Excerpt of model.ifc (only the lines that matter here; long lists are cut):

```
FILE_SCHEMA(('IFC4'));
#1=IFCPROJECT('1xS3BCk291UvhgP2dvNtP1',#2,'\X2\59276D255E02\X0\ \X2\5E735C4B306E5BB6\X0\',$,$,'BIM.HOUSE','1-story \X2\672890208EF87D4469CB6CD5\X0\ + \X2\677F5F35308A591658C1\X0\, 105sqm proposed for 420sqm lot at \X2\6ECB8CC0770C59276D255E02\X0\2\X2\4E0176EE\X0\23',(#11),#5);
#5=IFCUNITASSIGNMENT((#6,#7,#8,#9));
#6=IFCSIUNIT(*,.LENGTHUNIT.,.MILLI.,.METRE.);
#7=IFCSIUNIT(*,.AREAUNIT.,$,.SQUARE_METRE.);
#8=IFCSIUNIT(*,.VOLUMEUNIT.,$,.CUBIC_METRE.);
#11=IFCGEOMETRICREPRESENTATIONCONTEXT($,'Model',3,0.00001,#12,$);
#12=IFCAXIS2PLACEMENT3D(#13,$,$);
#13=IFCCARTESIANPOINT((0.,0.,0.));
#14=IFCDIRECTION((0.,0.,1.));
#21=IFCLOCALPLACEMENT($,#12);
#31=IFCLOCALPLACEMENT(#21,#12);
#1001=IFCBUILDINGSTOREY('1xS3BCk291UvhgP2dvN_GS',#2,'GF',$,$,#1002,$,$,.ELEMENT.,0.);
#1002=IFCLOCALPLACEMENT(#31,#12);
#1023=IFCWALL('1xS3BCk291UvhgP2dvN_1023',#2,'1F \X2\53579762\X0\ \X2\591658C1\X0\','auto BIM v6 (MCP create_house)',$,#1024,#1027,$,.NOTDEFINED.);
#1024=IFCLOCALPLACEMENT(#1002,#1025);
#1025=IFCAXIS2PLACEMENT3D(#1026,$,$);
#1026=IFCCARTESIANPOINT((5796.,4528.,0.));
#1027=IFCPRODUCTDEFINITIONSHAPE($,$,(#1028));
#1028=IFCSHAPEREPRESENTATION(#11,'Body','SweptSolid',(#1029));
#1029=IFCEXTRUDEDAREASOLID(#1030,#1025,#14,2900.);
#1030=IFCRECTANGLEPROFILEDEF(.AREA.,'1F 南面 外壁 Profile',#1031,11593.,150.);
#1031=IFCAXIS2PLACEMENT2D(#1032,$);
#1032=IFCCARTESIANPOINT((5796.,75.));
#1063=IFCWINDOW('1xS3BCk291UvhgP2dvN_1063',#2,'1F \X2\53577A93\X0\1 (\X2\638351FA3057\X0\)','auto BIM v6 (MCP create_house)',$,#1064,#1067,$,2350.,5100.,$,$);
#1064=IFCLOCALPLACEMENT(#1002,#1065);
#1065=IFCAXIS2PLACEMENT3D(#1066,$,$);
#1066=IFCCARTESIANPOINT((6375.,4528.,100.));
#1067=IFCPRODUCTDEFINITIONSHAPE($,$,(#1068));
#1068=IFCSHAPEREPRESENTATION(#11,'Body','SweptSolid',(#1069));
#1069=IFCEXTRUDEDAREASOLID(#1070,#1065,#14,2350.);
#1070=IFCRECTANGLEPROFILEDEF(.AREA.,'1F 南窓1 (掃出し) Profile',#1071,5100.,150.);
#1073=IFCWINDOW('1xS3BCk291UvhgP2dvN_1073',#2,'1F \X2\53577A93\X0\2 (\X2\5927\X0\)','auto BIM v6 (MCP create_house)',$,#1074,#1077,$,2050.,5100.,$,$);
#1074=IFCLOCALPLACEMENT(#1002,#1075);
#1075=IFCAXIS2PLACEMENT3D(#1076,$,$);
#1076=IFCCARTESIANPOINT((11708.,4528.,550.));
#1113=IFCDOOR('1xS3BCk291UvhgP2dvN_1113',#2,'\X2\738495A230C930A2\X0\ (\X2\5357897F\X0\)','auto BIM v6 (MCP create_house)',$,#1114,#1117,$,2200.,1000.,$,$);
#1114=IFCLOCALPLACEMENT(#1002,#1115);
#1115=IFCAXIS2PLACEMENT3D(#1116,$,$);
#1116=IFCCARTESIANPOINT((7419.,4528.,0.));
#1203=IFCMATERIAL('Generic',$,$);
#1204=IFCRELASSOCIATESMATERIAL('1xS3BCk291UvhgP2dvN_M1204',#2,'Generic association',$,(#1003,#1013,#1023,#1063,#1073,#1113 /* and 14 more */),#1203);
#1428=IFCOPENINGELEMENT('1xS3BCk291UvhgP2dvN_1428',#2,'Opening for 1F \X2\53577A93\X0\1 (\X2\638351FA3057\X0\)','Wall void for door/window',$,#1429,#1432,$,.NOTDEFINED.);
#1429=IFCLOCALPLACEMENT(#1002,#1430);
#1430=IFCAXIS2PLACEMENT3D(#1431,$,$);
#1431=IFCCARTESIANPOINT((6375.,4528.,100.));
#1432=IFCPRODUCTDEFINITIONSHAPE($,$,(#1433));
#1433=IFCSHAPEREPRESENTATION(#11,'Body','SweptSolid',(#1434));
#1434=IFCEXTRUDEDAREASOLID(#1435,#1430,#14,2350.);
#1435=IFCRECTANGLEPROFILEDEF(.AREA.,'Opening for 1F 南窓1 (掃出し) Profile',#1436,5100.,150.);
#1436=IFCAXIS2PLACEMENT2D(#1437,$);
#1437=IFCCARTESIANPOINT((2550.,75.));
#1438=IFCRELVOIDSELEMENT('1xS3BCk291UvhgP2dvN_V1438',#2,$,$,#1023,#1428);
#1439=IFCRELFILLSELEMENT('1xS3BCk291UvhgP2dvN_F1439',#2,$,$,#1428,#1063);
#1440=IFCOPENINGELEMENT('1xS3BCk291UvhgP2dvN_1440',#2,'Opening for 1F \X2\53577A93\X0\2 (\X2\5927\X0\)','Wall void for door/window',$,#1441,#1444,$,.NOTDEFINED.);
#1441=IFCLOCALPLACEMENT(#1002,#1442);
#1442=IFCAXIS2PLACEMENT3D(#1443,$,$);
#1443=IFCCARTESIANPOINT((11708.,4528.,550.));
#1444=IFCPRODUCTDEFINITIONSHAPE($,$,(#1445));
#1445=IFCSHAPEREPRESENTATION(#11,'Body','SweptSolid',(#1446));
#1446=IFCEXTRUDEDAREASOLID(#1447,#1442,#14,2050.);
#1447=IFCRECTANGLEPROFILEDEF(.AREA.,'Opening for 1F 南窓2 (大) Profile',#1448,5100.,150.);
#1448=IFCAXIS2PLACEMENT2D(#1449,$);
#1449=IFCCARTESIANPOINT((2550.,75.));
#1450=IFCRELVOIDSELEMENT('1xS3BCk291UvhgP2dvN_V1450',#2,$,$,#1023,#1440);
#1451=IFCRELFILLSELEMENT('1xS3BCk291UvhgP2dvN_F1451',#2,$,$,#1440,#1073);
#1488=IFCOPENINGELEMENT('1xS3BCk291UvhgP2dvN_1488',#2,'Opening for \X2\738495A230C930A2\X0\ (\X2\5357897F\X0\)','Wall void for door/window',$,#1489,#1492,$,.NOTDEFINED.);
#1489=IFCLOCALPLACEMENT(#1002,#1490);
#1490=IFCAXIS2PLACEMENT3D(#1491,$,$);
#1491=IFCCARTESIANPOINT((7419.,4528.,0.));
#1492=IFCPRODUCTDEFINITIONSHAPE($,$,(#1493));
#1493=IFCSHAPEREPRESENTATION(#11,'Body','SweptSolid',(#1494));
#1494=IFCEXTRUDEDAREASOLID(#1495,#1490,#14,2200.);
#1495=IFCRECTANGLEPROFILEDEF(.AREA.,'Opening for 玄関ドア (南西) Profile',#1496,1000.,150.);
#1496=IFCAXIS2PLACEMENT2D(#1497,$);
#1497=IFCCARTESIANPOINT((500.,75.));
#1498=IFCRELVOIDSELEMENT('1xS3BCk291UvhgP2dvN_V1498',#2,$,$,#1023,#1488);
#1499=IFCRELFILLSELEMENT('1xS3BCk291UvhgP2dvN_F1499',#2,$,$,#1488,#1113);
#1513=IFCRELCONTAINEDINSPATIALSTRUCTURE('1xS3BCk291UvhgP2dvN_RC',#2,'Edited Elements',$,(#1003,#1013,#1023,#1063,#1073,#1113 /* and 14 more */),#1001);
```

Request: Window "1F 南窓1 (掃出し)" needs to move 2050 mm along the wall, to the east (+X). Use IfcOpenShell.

```python
import ifcopenshell
import ifcopenshell.api.geometry
import ifcopenshell.util.placement
import ifcopenshell.util.unit

model = ifcopenshell.open("model.ifc")
unit_scale = ifcopenshell.util.unit.calculate_unit_scale(model)

window = model.by_id(1063)
opening = window.FillsVoids[0].RelatingOpeningElement
wall = opening.VoidsElements[0].RelatingBuildingElement

wall_matrix = ifcopenshell.util.placement.get_local_placement(wall.ObjectPlacement)
shift = wall_matrix[:3, 0] * 2.05 / unit_scale
before = ifcopenshell.util.placement.get_local_placement(window.ObjectPlacement)[:3, 3].copy()

# The window is not placed relative to its opening, so move both.
for product in (opening, window):
    matrix = ifcopenshell.util.placement.get_local_placement(product.ObjectPlacement)
    matrix[:3, 3] += shift
    ifcopenshell.api.geometry.edit_object_placement(model, product=product, matrix=matrix, is_si=False)

after = ifcopenshell.util.placement.get_local_placement(window.ObjectPlacement)[:3, 3]
print("window moved by", (after - before).round(3) + 0.0)

model.write("model_edited.ifc")
```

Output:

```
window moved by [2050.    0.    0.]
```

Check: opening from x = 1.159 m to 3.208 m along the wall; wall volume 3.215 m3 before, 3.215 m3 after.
